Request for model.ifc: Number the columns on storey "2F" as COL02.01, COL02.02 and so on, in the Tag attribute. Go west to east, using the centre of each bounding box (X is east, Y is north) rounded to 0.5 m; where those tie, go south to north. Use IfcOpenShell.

First a look at what the model holds.

```python
import ifcopenshell
import ifcopenshell.util.element
import ifcopenshell.util.placement

model = ifcopenshell.open("model.ifc")
print(model.schema)
storey = next(s for s in model.by_type("IfcBuildingStorey") if s.Name == "2F")
columns = [e for e in ifcopenshell.util.element.get_decomposition(storey) if e.is_a("IfcColumn")]
for e in sorted(columns, key=lambda e: e.id()):
    origin = ifcopenshell.util.placement.get_local_placement(e.ObjectPlacement)[:3, 3]
    print(e.id(), e.Tag, e.Name, origin.round(2) + 0.0, sep=" | ")
```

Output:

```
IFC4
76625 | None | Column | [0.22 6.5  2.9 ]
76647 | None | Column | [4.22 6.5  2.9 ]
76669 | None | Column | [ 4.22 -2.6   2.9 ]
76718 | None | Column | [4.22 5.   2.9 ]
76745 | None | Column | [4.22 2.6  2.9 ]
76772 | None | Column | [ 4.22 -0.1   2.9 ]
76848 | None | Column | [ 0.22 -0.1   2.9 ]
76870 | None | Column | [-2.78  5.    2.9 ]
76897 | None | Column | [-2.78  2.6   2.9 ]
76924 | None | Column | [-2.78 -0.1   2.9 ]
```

```python
import ifcopenshell
import ifcopenshell.geom
import ifcopenshell.util.element
import ifcopenshell.util.shape

model = ifcopenshell.open("model.ifc")
settings = ifcopenshell.geom.settings()
settings.set("use-world-coords", True)


def centre(element):
    shape = ifcopenshell.geom.create_shape(settings, element)
    return ifcopenshell.util.shape.get_bbox_centroid(shape.geometry)


storey = next(s for s in model.by_type("IfcBuildingStorey") if s.Name == "2F")
columns = [e for e in ifcopenshell.util.element.get_decomposition(storey) if e.is_a("IfcColumn")]

# Insertion points can sit at a corner or the storey origin, so sort by the geometry (in metres).
centres = {e: centre(e) for e in columns}
columns.sort(key=lambda e: (round(centres[e][0] / 0.5), centres[e][1]))

for i, e in enumerate(columns, start=1):
    number = f"COL02.{i:02d}"
    e.Tag = number
    print(e.id(), number)

model.write("model_updated.ifc")
```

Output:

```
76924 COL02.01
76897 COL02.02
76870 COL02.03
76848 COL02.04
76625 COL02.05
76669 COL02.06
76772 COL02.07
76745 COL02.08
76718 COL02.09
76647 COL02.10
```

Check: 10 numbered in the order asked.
